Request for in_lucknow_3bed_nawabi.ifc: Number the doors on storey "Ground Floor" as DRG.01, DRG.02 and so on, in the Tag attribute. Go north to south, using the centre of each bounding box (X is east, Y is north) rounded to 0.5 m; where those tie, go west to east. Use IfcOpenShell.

First a look at what the model holds.

```python
import ifcopenshell
import ifcopenshell.util.element
import ifcopenshell.util.placement

model = ifcopenshell.open("in_lucknow_3bed_nawabi.ifc")
print(model.schema)
storey = next(s for s in model.by_type("IfcBuildingStorey") if s.Name == "Ground Floor")
doors = [e for e in ifcopenshell.util.element.get_decomposition(storey) if e.is_a("IfcDoor")]
for e in sorted(doors, key=lambda e: e.id()):
    origin = ifcopenshell.util.placement.get_local_placement(e.ObjectPlacement)[:3, 3]
    print(e.id(), e.Tag, e.Name, origin.round(2) + 0.0, sep=" | ")
```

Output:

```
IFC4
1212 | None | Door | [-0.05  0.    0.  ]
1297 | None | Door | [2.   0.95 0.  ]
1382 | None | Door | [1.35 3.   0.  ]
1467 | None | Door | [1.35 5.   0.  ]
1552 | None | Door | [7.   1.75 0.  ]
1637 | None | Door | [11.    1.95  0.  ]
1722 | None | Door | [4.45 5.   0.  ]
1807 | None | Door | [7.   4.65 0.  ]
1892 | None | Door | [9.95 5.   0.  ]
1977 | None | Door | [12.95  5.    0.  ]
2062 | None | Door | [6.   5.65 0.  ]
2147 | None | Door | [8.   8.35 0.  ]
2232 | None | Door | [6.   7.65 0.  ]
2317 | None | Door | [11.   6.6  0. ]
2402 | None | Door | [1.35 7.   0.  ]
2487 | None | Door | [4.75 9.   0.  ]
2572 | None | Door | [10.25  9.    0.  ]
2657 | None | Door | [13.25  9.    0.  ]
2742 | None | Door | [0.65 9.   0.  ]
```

```python
import ifcopenshell
import ifcopenshell.geom
import ifcopenshell.util.element
import ifcopenshell.util.shape

model = ifcopenshell.open("in_lucknow_3bed_nawabi.ifc")
settings = ifcopenshell.geom.settings()
settings.set("use-world-coords", True)


def centre(element):
    shape = ifcopenshell.geom.create_shape(settings, element)
    return ifcopenshell.util.shape.get_bbox_centroid(shape.geometry)


storey = next(s for s in model.by_type("IfcBuildingStorey") if s.Name == "Ground Floor")
doors = [e for e in ifcopenshell.util.element.get_decomposition(storey) if e.is_a("IfcDoor")]

# Insertion points can sit at a corner or the storey origin, so sort by the geometry (in metres).
centres = {e: centre(e) for e in doors}
doors.sort(key=lambda e: (-round(centres[e][1] / 0.5), centres[e][0]))

for i, e in enumerate(doors, start=1):
    number = f"DRG.{i:02d}"
    e.Tag = number
    print(e.id(), number)

model.write("in_lucknow_3bed_nawabi-out.ifc")
```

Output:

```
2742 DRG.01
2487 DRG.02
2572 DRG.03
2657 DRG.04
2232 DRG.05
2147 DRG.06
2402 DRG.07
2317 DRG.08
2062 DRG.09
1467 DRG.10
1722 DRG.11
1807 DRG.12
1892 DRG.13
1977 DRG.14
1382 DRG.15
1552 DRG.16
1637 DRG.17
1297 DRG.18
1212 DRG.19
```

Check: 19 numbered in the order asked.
